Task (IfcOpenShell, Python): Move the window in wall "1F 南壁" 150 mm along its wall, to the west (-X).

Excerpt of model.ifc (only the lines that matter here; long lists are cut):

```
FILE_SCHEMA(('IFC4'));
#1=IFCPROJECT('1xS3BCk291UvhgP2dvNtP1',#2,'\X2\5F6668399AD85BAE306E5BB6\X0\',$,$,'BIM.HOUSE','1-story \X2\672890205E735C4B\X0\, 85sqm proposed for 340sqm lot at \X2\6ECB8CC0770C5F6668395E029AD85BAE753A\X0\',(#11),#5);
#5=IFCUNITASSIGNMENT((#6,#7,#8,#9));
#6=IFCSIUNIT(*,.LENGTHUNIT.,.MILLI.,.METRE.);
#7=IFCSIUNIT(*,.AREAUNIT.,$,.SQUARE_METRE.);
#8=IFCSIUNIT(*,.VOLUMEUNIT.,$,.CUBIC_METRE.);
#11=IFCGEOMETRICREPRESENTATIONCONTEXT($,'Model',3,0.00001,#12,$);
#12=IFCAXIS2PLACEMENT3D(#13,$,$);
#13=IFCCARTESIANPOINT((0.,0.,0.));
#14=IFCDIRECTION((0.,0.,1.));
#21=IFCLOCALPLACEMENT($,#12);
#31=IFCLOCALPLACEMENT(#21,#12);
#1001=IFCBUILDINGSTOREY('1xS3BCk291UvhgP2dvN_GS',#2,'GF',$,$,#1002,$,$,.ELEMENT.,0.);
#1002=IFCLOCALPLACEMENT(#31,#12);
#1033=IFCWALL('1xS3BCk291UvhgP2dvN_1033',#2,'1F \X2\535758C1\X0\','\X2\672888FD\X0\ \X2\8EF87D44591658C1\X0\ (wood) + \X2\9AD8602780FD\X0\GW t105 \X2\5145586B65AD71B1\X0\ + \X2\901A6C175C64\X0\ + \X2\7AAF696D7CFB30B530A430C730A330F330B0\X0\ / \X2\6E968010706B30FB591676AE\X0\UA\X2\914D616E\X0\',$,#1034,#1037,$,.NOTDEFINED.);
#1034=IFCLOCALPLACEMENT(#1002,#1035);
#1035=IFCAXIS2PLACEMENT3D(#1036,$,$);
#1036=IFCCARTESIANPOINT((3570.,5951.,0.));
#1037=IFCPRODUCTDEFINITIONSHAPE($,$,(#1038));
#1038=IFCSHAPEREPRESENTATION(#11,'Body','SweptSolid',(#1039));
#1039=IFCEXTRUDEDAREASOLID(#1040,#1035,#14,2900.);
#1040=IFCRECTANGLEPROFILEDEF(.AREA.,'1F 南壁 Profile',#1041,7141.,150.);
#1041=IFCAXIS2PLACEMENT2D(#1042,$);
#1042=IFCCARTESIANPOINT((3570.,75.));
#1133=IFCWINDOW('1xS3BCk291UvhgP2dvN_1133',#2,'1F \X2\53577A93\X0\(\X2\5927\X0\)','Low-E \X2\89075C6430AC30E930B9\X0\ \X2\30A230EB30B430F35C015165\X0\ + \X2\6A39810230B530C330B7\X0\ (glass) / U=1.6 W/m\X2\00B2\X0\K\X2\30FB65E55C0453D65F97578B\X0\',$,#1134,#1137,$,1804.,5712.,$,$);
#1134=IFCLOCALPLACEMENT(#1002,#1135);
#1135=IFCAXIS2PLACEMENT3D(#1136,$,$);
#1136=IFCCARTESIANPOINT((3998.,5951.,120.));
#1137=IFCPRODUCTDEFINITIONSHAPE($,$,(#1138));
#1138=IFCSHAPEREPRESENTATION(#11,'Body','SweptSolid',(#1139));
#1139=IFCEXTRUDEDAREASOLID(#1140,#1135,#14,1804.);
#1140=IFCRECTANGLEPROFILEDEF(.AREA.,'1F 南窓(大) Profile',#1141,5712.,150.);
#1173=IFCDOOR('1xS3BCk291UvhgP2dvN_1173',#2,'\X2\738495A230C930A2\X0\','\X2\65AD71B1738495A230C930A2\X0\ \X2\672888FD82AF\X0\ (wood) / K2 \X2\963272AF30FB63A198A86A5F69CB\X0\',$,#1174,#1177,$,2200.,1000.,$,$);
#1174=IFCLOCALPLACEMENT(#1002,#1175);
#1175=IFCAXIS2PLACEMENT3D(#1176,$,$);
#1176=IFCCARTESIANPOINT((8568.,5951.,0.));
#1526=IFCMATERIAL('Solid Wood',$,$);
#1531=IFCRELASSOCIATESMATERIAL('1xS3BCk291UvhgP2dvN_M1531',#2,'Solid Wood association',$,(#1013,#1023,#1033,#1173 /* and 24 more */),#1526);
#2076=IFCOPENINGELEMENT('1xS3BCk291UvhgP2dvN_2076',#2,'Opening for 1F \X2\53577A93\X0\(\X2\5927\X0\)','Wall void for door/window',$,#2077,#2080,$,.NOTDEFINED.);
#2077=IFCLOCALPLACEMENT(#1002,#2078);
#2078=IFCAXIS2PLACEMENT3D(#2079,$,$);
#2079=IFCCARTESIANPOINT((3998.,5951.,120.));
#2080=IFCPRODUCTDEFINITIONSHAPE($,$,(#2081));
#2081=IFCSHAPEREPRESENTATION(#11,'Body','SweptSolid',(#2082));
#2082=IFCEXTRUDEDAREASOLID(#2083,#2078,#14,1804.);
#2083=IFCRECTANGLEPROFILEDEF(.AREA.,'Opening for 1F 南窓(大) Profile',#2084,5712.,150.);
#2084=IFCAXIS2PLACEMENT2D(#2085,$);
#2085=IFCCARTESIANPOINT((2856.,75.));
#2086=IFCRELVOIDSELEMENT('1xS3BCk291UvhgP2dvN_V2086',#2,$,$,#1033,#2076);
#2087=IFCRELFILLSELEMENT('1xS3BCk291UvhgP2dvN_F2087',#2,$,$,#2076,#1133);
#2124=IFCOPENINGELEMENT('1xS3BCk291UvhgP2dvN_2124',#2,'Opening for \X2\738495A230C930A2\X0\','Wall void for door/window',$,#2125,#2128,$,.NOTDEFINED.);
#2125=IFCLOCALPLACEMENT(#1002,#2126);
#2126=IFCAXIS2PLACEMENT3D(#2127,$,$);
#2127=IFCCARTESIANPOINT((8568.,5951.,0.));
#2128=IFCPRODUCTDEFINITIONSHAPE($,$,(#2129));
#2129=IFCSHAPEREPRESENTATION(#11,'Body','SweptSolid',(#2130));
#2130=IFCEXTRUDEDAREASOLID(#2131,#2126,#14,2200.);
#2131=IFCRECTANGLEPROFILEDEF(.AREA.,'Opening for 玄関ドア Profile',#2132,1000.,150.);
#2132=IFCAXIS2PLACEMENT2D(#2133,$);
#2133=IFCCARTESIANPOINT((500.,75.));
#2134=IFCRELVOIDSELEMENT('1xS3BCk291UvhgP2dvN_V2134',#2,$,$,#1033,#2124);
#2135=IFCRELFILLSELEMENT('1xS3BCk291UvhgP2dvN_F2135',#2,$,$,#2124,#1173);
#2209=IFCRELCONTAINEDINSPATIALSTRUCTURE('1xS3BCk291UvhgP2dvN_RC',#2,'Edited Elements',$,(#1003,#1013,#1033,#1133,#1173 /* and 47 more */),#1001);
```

```python
import ifcopenshell
import ifcopenshell.api.geometry
import ifcopenshell.util.placement
import ifcopenshell.util.unit

model = ifcopenshell.open("model.ifc")
unit_scale = ifcopenshell.util.unit.calculate_unit_scale(model)

window = model.by_guid("1xS3BCk291UvhgP2dvN_1133")
opening = window.FillsVoids[0].RelatingOpeningElement
wall = opening.VoidsElements[0].RelatingBuildingElement

wall_matrix = ifcopenshell.util.placement.get_local_placement(wall.ObjectPlacement)
shift = wall_matrix[:3, 0] * -0.15 / unit_scale
before = ifcopenshell.util.placement.get_local_placement(window.ObjectPlacement)[:3, 3].copy()

# The window is not placed relative to its opening, so move both.
for product in (opening, window):
    matrix = ifcopenshell.util.placement.get_local_placement(product.ObjectPlacement)
    matrix[:3, 3] += shift
    ifcopenshell.api.geometry.edit_object_placement(model, product=product, matrix=matrix, is_si=False)

after = ifcopenshell.util.placement.get_local_placement(window.ObjectPlacement)[:3, 3]
print("window moved by", (after - before).round(3) + 0.0)

model.write("model-out.ifc")
```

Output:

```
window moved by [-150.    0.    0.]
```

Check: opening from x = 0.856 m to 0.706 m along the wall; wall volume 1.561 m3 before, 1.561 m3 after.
